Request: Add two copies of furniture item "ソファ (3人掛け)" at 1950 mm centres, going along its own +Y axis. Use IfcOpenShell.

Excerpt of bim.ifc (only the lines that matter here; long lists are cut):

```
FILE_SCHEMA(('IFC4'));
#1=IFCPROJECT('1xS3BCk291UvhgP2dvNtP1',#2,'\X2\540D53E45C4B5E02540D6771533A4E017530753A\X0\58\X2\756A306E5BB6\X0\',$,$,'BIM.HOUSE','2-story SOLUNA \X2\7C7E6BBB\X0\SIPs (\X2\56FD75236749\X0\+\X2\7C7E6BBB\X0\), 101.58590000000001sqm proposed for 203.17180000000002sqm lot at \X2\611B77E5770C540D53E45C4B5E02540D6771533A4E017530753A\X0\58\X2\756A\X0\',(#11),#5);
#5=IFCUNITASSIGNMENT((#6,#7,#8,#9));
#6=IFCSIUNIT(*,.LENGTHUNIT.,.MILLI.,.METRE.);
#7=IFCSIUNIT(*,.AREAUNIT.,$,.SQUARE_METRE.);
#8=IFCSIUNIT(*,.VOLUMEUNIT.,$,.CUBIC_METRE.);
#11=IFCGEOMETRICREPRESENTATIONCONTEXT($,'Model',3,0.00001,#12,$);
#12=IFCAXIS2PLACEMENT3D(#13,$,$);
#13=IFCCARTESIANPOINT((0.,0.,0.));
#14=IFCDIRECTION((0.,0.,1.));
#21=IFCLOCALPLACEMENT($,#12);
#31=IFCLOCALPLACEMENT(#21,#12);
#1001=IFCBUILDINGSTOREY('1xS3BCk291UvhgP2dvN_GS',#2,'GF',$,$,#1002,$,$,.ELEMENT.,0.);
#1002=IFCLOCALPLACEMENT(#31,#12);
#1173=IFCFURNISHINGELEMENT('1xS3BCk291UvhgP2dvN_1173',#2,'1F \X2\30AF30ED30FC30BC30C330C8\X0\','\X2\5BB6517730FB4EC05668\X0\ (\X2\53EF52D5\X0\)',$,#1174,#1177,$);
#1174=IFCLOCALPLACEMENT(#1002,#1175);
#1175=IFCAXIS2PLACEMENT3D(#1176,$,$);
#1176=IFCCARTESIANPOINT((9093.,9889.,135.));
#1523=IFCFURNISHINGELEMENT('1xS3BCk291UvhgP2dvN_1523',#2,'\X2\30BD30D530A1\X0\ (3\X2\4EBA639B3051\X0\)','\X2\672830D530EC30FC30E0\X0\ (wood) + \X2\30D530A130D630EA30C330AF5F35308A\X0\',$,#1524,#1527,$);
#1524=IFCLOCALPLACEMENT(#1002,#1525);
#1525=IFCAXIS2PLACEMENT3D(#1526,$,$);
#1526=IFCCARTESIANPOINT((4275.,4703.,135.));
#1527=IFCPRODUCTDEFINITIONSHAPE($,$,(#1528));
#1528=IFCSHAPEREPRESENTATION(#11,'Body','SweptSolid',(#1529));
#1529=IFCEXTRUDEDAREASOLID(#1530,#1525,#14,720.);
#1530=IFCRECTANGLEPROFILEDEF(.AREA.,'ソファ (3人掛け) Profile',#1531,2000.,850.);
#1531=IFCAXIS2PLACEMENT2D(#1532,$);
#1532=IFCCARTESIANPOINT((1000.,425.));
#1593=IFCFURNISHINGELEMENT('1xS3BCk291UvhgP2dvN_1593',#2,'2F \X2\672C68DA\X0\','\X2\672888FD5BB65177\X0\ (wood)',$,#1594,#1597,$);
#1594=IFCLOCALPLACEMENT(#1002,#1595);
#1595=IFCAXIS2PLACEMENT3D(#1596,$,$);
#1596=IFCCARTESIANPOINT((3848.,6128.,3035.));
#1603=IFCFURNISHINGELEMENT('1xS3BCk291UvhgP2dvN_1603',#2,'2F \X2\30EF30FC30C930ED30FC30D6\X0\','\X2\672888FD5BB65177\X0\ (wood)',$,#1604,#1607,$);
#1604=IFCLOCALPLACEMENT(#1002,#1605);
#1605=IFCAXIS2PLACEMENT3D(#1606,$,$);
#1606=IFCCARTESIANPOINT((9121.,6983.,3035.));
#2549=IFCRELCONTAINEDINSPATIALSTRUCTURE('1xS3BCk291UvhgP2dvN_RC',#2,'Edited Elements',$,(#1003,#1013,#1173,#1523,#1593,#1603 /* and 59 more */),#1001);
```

```python
import ifcopenshell
import ifcopenshell.api.geometry
import ifcopenshell.api.root
import ifcopenshell.util.element
import ifcopenshell.util.placement

model = ifcopenshell.open("bim.ifc")


def reuse_history(source, copy):
    """copy_class also copies each property set's owner history, people and application; keep the originals."""
    for rel in copy.IsDefinedBy:
        if rel.is_a("IfcRelDefinesByProperties") and (history := rel.RelatingPropertyDefinition.OwnerHistory):
            rel.RelatingPropertyDefinition.OwnerHistory = source.OwnerHistory
            ifcopenshell.util.element.remove_deep2(model, history)


source = model.by_guid("1xS3BCk291UvhgP2dvN_1523")
base = ifcopenshell.util.placement.get_local_placement(source.ObjectPlacement)
step = base[:3, 1] * 1950.0

for i in range(1, 3):
    copy = ifcopenshell.api.root.copy_class(model, product=source)
    copy.Representation = ifcopenshell.util.element.copy_deep(
        model, source.Representation, exclude=["IfcGeometricRepresentationContext", "IfcRepresentationMap"]
    )
    reuse_history(source, copy)
    matrix = base.copy()
    matrix[:3, 3] += i * step
    print("added at", matrix[:3, 3].round(3) + 0.0)
    ifcopenshell.api.geometry.edit_object_placement(model, product=copy, matrix=matrix, is_si=False)

model.write("bim_rev.ifc")
```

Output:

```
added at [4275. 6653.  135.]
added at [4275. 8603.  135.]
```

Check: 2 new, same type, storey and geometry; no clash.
